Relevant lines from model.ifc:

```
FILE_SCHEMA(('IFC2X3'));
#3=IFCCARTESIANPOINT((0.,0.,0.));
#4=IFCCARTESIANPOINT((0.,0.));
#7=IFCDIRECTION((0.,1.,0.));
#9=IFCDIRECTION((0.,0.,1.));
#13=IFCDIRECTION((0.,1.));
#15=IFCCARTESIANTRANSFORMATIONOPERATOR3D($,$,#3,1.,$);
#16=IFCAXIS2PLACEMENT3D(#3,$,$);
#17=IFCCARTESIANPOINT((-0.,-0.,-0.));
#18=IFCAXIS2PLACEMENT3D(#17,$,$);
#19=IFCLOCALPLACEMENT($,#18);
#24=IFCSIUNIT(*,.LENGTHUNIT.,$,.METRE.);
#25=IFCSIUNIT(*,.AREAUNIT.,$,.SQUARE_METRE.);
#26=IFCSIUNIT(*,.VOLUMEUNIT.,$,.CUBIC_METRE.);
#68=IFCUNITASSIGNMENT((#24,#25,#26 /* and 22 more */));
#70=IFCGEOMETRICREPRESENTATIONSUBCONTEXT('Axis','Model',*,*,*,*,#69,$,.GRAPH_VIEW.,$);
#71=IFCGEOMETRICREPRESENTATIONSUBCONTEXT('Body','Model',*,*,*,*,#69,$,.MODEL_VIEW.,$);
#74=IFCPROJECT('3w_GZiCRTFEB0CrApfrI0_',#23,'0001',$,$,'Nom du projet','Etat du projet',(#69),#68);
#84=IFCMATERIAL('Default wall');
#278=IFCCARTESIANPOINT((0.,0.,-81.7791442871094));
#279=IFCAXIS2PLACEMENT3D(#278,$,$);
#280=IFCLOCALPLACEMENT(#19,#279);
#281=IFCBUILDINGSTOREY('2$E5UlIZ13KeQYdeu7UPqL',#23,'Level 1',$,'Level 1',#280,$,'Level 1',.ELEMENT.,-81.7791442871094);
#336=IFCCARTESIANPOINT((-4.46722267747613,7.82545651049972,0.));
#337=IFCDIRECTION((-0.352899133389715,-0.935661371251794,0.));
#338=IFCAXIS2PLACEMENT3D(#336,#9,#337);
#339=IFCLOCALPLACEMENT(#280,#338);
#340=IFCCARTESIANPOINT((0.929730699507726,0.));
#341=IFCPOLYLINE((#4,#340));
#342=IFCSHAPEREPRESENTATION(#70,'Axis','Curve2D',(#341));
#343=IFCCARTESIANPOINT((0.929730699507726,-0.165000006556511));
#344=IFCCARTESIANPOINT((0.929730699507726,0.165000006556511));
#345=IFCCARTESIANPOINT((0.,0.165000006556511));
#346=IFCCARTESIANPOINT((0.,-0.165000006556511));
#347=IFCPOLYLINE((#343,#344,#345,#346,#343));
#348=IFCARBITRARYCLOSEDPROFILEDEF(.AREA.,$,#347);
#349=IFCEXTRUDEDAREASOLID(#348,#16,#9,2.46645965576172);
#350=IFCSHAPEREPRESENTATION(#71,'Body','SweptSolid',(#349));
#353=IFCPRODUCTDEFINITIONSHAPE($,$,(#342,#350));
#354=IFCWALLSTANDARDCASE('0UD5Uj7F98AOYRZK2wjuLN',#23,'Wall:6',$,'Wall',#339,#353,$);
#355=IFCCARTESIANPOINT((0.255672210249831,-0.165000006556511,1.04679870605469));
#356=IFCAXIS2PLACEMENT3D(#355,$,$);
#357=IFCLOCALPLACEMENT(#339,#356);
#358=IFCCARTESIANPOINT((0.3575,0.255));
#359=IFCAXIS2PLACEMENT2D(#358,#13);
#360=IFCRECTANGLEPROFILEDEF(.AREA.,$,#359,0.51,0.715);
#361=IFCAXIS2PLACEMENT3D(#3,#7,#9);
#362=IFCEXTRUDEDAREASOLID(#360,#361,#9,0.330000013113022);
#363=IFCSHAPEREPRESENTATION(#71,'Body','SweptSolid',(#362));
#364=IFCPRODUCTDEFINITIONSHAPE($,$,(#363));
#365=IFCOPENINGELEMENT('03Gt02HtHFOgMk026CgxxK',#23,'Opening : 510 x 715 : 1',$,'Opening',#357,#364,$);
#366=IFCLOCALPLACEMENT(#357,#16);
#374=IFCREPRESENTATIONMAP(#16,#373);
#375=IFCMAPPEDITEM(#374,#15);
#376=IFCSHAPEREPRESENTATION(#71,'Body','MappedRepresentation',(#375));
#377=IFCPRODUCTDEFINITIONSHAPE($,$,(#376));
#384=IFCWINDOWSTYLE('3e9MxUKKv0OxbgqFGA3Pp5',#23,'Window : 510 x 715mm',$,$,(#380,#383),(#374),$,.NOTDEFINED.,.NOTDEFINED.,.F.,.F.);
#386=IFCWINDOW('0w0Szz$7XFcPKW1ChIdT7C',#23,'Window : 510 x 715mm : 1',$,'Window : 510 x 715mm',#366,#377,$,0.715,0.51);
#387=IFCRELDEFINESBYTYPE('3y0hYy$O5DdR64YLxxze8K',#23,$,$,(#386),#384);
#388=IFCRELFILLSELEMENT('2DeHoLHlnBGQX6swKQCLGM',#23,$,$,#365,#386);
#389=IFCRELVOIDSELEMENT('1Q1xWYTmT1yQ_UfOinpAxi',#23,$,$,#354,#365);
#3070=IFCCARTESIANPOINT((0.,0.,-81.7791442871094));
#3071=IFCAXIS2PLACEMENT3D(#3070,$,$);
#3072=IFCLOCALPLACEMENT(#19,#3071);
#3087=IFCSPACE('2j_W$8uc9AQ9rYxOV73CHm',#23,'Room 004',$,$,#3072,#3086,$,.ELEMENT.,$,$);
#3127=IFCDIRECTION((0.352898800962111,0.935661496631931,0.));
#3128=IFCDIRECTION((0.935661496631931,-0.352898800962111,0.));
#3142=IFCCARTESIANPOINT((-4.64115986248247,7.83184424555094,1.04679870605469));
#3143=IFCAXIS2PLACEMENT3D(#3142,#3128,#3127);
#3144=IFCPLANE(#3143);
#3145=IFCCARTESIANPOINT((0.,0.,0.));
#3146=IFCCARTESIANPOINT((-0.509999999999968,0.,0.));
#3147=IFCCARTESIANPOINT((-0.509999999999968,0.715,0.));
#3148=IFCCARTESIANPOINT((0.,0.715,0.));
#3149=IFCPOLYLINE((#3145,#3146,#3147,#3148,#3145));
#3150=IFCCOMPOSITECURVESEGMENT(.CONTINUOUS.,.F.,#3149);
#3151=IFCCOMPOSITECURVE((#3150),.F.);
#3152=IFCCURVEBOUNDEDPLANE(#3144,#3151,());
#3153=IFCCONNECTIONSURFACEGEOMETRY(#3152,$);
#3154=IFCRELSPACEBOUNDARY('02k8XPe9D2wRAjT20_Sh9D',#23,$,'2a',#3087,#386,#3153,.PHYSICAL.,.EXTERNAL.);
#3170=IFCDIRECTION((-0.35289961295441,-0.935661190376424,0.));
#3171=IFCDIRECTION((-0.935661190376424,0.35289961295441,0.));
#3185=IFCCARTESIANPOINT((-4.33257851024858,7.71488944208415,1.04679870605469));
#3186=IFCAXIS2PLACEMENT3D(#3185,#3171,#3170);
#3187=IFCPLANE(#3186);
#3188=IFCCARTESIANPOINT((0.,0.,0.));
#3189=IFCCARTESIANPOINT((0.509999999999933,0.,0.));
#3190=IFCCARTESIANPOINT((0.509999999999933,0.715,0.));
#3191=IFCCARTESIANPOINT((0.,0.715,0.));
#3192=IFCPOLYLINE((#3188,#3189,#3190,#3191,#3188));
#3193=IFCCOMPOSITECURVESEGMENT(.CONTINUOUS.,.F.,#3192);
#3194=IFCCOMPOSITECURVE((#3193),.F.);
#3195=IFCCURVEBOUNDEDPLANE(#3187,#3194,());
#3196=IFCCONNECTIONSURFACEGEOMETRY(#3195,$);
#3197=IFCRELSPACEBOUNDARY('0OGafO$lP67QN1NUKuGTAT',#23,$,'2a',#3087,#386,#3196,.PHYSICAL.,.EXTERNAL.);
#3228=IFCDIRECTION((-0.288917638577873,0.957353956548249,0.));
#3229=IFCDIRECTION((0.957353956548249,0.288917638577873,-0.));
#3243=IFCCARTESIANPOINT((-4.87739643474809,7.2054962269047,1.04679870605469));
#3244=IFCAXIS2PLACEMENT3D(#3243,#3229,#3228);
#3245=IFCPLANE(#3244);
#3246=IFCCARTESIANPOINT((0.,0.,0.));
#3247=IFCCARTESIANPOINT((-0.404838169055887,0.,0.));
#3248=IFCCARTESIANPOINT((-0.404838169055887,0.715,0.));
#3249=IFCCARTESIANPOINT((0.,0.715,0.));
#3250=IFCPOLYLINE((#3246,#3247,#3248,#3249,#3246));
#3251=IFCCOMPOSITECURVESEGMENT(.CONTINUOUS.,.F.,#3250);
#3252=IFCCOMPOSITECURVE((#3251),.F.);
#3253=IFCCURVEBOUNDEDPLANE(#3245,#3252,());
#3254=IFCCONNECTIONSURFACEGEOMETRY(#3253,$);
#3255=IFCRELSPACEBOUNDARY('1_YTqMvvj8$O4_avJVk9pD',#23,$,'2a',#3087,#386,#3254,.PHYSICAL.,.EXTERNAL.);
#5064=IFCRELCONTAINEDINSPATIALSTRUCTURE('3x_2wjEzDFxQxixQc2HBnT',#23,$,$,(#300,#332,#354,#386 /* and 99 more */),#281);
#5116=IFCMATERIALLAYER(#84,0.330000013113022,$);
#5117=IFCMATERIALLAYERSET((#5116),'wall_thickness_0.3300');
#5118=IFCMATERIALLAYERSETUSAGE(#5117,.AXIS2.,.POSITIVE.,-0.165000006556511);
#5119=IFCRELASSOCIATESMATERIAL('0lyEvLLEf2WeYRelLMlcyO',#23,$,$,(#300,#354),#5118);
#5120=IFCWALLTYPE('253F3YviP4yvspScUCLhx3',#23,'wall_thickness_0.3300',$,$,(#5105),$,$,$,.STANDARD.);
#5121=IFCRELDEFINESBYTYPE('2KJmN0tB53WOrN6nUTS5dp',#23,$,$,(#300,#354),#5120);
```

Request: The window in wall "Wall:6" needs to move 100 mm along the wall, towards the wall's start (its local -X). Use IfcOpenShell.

```python
import numpy as np
import ifcopenshell
import ifcopenshell.api.geometry
import ifcopenshell.util.placement
import ifcopenshell.util.unit

model = ifcopenshell.open("model.ifc")
unit_scale = ifcopenshell.util.unit.calculate_unit_scale(model)

window = model.by_guid("0w0Szz$7XFcPKW1ChIdT7C")
opening = window.FillsVoids[0].RelatingOpeningElement
wall = opening.VoidsElements[0].RelatingBuildingElement

wall_matrix = ifcopenshell.util.placement.get_local_placement(wall.ObjectPlacement)
shift = wall_matrix[:3, 0] * -0.1 / unit_scale
before = ifcopenshell.util.placement.get_local_placement(window.ObjectPlacement)[:3, 3].copy()

# The window is placed relative to its opening, so it follows when the opening moves.
matrix = ifcopenshell.util.placement.get_local_placement(opening.ObjectPlacement)
matrix[:3, 3] += shift
ifcopenshell.api.geometry.edit_object_placement(
    model, product=opening, matrix=matrix, is_si=False, should_transform_children=True
)

# Space boundary surfaces are stored in each space's coordinates; move them too.
for rel in window.ProvidesBoundaries:
    if not rel.ConnectionGeometry:
        continue
    surface = rel.ConnectionGeometry.SurfaceOnRelatingElement.BasisSurface
    space_matrix = ifcopenshell.util.placement.get_local_placement(rel.RelatingSpace.ObjectPlacement)
    point = np.array(surface.Position.Location.Coordinates) + space_matrix[:3, :3].T @ shift
    surface.Position = model.createIfcAxis2Placement3D(
        model.createIfcCartesianPoint(point.tolist()), surface.Position.Axis, surface.Position.RefDirection
    )

after = ifcopenshell.util.placement.get_local_placement(window.ObjectPlacement)[:3, 3]
print("window moved by", (after - before).round(3) + 0.0)

model.write("model-out.ifc")
```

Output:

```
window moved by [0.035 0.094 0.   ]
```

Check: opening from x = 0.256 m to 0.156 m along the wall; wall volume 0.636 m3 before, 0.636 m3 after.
